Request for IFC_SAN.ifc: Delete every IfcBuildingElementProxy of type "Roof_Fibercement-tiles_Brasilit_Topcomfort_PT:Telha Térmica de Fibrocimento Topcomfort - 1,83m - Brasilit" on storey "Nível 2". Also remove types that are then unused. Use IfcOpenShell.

First a look at what the model holds.

```python
import ifcopenshell
import ifcopenshell.util.element

model = ifcopenshell.open("IFC_SAN.ifc")
print(model.schema)
storey = next(s for s in model.by_type("IfcBuildingStorey") if s.Name == "Nível 2")
proxies = [e for e in ifcopenshell.util.element.get_decomposition(storey) if e.is_a("IfcBuildingElementProxy")]
seen = {}
for e in proxies:
    element_type = ifcopenshell.util.element.get_type(e)
    name = element_type.Name if element_type not in (None, e) else None
    seen[name] = seen.get(name, 0) + 1
for name, count in sorted(seen.items(), key=str):
    print(count, "x", name)
```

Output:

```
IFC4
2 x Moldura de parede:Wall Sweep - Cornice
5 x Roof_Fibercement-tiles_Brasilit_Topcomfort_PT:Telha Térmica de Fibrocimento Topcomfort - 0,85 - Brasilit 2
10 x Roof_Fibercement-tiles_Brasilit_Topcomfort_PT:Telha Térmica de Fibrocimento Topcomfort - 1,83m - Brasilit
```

```python
import ifcopenshell
import ifcopenshell.api.root
import ifcopenshell.util.element

model = ifcopenshell.open("IFC_SAN.ifc")

storey = next(s for s in model.by_type("IfcBuildingStorey") if s.Name == "Nível 2")
proxies = [e for e in ifcopenshell.util.element.get_decomposition(storey) if e.is_a("IfcBuildingElementProxy")]
targets = [e for e in proxies if (t := ifcopenshell.util.element.get_type(e)) not in (None, e) and t.Name == "Roof_Fibercement-tiles_Brasilit_Topcomfort_PT:Telha Térmica de Fibrocimento Topcomfort - 1,83m - Brasilit"]
types = {ifcopenshell.util.element.get_type(e) for e in targets} - {None, *targets}

for e in targets:
    ifcopenshell.api.root.remove_product(model, product=e)
print(len(targets), "removed")

unused = [t for t in types if not ifcopenshell.util.element.get_types(t)]
for t in unused:
    ifcopenshell.api.root.remove_product(model, product=t)
print(len(unused), "unused types removed")

model.write("IFC_SAN_updated.ifc")
```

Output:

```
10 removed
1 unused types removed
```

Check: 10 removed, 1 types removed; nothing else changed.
